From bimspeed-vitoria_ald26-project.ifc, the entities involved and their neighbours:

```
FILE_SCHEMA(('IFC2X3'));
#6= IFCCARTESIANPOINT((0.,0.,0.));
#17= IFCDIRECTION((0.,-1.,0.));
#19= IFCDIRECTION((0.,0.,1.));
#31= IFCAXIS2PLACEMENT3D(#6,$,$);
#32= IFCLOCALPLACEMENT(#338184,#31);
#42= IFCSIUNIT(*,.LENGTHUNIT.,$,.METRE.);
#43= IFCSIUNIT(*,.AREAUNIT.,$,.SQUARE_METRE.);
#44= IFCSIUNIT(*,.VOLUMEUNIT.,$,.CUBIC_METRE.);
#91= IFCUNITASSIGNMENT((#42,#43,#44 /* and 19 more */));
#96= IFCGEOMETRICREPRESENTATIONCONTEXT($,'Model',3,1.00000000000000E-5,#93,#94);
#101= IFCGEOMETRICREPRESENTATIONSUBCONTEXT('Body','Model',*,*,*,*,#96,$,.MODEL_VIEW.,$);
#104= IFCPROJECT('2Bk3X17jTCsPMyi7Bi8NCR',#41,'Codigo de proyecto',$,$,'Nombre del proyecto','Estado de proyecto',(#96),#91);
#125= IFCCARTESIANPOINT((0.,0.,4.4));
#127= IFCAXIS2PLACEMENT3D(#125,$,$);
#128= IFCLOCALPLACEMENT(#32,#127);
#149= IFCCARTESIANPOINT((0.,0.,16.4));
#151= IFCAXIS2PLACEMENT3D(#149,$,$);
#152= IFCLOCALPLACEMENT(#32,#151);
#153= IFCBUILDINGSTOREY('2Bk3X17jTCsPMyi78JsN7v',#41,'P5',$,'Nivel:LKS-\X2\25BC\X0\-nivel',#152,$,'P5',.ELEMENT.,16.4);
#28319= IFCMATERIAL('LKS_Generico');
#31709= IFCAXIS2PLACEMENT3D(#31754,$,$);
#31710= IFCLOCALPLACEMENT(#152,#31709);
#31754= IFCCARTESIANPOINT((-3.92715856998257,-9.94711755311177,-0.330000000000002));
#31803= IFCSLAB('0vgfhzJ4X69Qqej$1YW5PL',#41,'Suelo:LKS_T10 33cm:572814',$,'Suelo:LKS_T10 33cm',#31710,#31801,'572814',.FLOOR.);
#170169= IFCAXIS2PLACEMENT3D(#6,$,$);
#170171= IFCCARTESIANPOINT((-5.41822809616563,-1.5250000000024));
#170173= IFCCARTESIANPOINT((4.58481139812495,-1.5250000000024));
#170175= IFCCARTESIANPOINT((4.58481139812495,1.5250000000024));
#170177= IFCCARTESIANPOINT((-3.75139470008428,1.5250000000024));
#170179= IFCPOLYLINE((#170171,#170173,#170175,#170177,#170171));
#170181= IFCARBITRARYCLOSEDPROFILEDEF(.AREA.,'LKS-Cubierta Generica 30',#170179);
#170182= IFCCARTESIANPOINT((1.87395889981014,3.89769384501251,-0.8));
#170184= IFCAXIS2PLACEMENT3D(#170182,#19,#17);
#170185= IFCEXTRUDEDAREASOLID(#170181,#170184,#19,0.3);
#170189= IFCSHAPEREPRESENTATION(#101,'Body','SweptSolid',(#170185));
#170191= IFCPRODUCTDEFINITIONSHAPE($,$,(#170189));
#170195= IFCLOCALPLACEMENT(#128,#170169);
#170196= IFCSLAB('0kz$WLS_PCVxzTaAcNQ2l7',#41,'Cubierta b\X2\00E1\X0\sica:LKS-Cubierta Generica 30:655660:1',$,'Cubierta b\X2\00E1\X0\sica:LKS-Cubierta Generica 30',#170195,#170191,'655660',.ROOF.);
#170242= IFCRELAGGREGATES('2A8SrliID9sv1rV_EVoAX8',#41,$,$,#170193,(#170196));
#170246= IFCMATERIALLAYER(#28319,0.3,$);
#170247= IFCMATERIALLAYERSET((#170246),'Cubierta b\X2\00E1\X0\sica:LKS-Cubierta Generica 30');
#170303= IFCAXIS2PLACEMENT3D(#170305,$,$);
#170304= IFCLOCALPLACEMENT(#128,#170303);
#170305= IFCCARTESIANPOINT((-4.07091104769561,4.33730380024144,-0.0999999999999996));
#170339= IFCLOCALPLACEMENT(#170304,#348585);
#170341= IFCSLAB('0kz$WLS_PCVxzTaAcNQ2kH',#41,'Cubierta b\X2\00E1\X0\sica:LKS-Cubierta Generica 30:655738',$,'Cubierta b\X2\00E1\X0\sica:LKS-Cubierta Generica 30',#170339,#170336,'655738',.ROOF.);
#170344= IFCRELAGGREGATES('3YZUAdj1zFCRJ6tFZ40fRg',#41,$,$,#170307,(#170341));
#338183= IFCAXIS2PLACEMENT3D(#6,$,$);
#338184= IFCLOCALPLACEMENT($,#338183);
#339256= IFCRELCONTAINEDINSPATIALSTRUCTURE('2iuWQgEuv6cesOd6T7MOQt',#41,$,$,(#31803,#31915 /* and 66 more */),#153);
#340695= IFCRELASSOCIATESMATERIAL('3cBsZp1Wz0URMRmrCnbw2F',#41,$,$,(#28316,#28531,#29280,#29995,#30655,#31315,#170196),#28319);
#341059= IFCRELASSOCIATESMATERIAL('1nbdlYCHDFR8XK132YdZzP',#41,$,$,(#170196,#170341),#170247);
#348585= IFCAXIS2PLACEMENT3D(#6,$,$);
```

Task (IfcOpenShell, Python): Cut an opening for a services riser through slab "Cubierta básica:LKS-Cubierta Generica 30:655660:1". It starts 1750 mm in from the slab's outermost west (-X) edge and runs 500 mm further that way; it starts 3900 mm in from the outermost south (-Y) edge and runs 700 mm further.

```python
import numpy as np
import ifcopenshell
import ifcopenshell.api.feature
import ifcopenshell.api.geometry
import ifcopenshell.api.root
import ifcopenshell.geom
import ifcopenshell.util.placement
import ifcopenshell.util.representation
import ifcopenshell.util.shape
import ifcopenshell.util.unit

model = ifcopenshell.open("bimspeed-vitoria_ald26-project.ifc")
unit_scale = ifcopenshell.util.unit.calculate_unit_scale(model)
settings = ifcopenshell.geom.settings()


def volume(element):
    """Net volume in cubic metres, openings subtracted."""
    shape = ifcopenshell.geom.create_shape(settings, element)
    return ifcopenshell.util.shape.get_volume(shape.geometry)


slab = model.by_guid("0kz$WLS_PCVxzTaAcNQ2l7")
before = volume(slab)

# Extent in the slab's own axes, in metres. The edges named are its -X and -Y sides.
slab_shape = ifcopenshell.geom.create_shape(settings, slab)
vertices = ifcopenshell.util.shape.get_vertices(slab_shape.geometry)
x_min, y_min, bottom = vertices.min(axis=0)
top = vertices[:, 2].max()

opening = ifcopenshell.api.root.create_entity(model, ifc_class="IfcOpeningElement", name="Services riser opening")
context = ifcopenshell.util.representation.get_context(model, "Model", "Body", "MODEL_VIEW")
width, depth = 0.5, 0.7
outline = [(0.0, 0.0), (width, 0.0), (width, depth), (0.0, depth), (0.0, 0.0)]
# Overshoot both faces by 50 mm so the cut is clean.
shape = ifcopenshell.api.geometry.add_slab_representation(
    model, context=context, depth=top - bottom + 0.1, polyline=outline
)
ifcopenshell.api.geometry.assign_representation(model, product=opening, representation=shape)

matrix = ifcopenshell.util.placement.get_local_placement(slab.ObjectPlacement)
matrix[:, 3] = matrix @ np.append(np.array([x_min + 1.75, y_min + 3.9, bottom - 0.05]) / unit_scale, 1.0)
ifcopenshell.api.geometry.edit_object_placement(model, product=opening, matrix=matrix, is_si=False)
ifcopenshell.api.feature.add_feature(model, feature=opening, element=slab)

after = volume(slab)

print(f"slab volume {before:.3f} -> {after:.3f} m3")

model.write("bimspeed-vitoria_ald26-project_updated.ifc")
```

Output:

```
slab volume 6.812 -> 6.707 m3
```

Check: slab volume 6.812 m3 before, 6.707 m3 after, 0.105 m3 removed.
